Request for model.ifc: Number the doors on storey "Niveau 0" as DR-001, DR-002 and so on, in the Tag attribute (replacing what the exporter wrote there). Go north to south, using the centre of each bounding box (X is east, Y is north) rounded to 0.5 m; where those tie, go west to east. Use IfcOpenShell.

First a look at what the model holds.

```python
import ifcopenshell
import ifcopenshell.util.element
import ifcopenshell.util.placement

model = ifcopenshell.open("model.ifc")
print(model.schema)
storey = next(s for s in model.by_type("IfcBuildingStorey") if s.Name == "Niveau 0")
doors = [e for e in ifcopenshell.util.element.get_decomposition(storey) if e.is_a("IfcDoor")]
for e in sorted(doors, key=lambda e: e.id()):
    origin = ifcopenshell.util.placement.get_local_placement(e.ObjectPlacement)[:3, 3]
    print(e.id(), e.Tag, e.Name, origin.round(2) + 0.0, sep=" | ")
```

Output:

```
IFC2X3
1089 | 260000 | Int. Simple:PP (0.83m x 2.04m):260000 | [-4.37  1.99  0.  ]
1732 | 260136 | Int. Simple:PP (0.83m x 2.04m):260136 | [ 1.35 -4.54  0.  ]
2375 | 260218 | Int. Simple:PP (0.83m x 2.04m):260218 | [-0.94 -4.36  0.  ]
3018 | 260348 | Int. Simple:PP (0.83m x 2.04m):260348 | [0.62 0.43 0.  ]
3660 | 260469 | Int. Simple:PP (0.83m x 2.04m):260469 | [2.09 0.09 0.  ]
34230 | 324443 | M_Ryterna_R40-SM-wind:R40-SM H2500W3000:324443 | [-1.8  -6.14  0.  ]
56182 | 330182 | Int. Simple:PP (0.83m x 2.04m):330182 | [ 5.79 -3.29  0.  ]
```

```python
import ifcopenshell
import ifcopenshell.geom
import ifcopenshell.util.element
import ifcopenshell.util.shape

model = ifcopenshell.open("model.ifc")
settings = ifcopenshell.geom.settings()
settings.set("use-world-coords", True)


def centre(element):
    shape = ifcopenshell.geom.create_shape(settings, element)
    return ifcopenshell.util.shape.get_bbox_centroid(shape.geometry)


storey = next(s for s in model.by_type("IfcBuildingStorey") if s.Name == "Niveau 0")
doors = [e for e in ifcopenshell.util.element.get_decomposition(storey) if e.is_a("IfcDoor")]

# Insertion points can sit at a corner or the storey origin, so sort by the geometry (in metres).
centres = {e: centre(e) for e in doors}
doors.sort(key=lambda e: (-round(centres[e][1] / 0.5), centres[e][0]))

for i, e in enumerate(doors, start=1):
    number = f"DR-0{i:02d}"
    e.Tag = number
    print(e.id(), number)

model.write("model_edited.ifc")
```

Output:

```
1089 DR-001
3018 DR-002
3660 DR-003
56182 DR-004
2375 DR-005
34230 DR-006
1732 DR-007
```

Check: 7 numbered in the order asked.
